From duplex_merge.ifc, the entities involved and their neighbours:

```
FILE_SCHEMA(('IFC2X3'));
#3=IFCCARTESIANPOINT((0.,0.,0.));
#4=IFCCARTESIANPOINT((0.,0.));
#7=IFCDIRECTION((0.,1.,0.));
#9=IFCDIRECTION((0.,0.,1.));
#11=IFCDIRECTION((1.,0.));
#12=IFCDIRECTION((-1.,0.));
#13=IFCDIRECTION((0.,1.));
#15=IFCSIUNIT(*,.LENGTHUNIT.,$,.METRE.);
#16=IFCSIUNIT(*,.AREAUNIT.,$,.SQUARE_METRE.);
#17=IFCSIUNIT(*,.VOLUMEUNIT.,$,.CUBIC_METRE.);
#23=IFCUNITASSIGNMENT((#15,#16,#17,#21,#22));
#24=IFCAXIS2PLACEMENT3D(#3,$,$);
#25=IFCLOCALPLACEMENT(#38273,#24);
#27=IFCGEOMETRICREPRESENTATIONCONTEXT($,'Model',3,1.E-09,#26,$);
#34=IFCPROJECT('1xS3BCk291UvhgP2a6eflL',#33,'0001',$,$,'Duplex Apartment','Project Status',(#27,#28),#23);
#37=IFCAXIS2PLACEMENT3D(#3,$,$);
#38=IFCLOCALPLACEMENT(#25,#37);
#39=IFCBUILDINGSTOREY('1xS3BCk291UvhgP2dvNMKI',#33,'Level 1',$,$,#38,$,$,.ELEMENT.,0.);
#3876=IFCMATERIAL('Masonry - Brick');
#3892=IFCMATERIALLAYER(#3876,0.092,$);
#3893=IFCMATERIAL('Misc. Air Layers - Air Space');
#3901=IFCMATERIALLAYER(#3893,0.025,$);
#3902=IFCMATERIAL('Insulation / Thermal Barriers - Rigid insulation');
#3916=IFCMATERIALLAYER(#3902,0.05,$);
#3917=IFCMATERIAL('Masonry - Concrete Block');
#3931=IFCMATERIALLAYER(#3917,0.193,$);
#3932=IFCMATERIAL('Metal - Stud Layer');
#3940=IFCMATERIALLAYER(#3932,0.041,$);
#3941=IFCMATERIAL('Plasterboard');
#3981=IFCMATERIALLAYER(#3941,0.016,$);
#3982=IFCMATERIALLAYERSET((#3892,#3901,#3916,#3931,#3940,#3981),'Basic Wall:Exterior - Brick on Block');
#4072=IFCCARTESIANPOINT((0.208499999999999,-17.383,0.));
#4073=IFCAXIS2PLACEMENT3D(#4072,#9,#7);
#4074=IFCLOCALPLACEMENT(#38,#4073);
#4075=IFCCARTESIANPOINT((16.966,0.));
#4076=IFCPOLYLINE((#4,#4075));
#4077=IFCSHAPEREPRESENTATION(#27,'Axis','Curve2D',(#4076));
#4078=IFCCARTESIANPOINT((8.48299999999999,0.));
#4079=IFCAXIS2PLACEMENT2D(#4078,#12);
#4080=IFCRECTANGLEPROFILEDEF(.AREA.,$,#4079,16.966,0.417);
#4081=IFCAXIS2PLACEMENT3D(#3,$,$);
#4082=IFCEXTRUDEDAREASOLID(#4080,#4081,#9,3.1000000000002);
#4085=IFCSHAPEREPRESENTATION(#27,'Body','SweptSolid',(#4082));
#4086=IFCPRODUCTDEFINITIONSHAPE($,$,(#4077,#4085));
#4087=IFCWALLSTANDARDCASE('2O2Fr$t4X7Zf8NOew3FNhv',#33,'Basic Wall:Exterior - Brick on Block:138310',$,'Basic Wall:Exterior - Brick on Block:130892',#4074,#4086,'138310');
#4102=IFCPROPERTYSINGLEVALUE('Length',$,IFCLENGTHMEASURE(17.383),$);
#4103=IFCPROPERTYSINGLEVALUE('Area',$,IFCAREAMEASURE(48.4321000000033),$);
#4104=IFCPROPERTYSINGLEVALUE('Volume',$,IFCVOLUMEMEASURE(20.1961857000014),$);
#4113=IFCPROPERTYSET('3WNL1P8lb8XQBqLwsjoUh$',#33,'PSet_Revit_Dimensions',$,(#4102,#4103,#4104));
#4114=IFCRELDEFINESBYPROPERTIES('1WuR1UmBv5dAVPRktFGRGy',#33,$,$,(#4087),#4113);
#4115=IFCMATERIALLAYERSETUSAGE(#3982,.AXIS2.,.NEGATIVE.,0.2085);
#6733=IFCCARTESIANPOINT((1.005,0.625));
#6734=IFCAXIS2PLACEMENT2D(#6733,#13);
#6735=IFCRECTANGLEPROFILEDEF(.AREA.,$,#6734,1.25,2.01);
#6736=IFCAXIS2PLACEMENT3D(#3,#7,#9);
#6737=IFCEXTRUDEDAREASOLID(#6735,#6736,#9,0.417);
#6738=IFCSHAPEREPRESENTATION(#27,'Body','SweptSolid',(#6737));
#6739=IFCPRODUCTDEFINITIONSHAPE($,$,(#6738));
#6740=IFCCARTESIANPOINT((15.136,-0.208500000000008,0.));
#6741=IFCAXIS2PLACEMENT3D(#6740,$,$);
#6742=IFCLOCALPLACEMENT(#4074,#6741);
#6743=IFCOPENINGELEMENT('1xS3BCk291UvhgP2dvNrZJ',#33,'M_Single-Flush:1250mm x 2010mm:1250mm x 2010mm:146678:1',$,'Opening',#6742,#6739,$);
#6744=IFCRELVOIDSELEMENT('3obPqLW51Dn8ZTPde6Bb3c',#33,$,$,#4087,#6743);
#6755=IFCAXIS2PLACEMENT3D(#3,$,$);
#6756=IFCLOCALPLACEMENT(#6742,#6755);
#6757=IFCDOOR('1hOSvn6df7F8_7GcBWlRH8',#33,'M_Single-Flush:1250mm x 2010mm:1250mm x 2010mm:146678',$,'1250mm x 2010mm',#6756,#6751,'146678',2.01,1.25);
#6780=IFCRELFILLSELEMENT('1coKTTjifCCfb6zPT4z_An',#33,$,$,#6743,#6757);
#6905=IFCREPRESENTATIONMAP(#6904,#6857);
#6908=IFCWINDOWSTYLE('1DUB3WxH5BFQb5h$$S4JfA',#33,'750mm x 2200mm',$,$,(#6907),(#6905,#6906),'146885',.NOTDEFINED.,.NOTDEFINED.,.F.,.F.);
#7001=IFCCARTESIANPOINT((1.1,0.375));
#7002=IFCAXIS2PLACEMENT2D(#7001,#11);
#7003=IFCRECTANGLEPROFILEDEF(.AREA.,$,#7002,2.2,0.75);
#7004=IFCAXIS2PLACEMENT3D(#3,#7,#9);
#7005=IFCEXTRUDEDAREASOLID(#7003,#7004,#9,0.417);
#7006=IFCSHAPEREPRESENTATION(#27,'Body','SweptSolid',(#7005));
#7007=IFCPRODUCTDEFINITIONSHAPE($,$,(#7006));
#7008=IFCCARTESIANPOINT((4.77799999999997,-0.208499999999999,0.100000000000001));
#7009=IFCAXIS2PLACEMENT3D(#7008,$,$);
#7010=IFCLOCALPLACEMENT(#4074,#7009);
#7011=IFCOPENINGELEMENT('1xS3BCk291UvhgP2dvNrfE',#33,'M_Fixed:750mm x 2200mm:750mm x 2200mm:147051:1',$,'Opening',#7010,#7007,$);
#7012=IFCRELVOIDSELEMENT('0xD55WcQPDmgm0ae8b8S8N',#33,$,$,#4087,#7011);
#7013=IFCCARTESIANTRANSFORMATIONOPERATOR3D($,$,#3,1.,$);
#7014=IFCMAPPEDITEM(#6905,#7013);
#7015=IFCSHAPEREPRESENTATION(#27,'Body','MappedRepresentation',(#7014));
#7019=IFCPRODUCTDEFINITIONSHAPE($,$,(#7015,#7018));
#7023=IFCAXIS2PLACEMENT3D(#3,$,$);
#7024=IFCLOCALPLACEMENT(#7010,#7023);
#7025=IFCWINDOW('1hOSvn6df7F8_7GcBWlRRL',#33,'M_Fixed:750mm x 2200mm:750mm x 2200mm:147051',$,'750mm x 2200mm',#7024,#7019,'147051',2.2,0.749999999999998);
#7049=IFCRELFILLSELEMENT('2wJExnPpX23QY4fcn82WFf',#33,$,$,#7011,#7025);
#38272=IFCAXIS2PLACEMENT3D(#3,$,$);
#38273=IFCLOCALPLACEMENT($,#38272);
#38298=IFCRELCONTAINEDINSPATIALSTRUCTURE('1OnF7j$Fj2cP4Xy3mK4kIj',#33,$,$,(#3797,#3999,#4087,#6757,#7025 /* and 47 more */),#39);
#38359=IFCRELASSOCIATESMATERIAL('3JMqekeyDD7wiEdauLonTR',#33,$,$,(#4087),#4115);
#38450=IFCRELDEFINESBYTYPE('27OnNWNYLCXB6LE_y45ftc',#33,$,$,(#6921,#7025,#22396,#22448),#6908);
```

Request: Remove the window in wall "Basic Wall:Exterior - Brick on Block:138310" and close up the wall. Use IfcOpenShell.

```python
import ifcopenshell
import ifcopenshell.api.feature
import ifcopenshell.api.pset
import ifcopenshell.api.root
import ifcopenshell.geom
import ifcopenshell.util.element
import ifcopenshell.util.shape
import ifcopenshell.util.unit

model = ifcopenshell.open("duplex_merge.ifc")
area_scale = ifcopenshell.util.unit.calculate_unit_scale(model, "AREAUNIT")
volume_scale = ifcopenshell.util.unit.calculate_unit_scale(model, "VOLUMEUNIT")
settings = ifcopenshell.geom.settings()


def volume(element):
    """Net volume in cubic metres, openings subtracted."""
    shape = ifcopenshell.geom.create_shape(settings, element)
    return ifcopenshell.util.shape.get_volume(shape.geometry)


window = model.by_id(7025)
opening = window.FillsVoids[0].RelatingOpeningElement
wall = opening.VoidsElements[0].RelatingBuildingElement
before = volume(wall)

ifcopenshell.api.root.remove_product(model, product=window)
ifcopenshell.api.feature.remove_feature(model, feature=opening)

after = volume(wall)
thickness = 0.417  # wall thickness in metres

# Update the wall's stored quantities.
pset = model.by_id(ifcopenshell.util.element.get_pset(wall, "PSet_Revit_Dimensions", should_inherit=False)["id"])
ifcopenshell.api.pset.edit_pset(model, pset=pset, properties={
    "Area": model.create_entity("IfcAreaMeasure", after / thickness / area_scale),
    "Volume": model.create_entity("IfcVolumeMeasure", after / volume_scale),
})

print(f"wall volume {before:.3f} -> {after:.3f} m3")

model.write("duplex_merge_edited.ifc")
```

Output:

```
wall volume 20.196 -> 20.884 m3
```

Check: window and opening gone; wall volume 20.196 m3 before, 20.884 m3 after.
